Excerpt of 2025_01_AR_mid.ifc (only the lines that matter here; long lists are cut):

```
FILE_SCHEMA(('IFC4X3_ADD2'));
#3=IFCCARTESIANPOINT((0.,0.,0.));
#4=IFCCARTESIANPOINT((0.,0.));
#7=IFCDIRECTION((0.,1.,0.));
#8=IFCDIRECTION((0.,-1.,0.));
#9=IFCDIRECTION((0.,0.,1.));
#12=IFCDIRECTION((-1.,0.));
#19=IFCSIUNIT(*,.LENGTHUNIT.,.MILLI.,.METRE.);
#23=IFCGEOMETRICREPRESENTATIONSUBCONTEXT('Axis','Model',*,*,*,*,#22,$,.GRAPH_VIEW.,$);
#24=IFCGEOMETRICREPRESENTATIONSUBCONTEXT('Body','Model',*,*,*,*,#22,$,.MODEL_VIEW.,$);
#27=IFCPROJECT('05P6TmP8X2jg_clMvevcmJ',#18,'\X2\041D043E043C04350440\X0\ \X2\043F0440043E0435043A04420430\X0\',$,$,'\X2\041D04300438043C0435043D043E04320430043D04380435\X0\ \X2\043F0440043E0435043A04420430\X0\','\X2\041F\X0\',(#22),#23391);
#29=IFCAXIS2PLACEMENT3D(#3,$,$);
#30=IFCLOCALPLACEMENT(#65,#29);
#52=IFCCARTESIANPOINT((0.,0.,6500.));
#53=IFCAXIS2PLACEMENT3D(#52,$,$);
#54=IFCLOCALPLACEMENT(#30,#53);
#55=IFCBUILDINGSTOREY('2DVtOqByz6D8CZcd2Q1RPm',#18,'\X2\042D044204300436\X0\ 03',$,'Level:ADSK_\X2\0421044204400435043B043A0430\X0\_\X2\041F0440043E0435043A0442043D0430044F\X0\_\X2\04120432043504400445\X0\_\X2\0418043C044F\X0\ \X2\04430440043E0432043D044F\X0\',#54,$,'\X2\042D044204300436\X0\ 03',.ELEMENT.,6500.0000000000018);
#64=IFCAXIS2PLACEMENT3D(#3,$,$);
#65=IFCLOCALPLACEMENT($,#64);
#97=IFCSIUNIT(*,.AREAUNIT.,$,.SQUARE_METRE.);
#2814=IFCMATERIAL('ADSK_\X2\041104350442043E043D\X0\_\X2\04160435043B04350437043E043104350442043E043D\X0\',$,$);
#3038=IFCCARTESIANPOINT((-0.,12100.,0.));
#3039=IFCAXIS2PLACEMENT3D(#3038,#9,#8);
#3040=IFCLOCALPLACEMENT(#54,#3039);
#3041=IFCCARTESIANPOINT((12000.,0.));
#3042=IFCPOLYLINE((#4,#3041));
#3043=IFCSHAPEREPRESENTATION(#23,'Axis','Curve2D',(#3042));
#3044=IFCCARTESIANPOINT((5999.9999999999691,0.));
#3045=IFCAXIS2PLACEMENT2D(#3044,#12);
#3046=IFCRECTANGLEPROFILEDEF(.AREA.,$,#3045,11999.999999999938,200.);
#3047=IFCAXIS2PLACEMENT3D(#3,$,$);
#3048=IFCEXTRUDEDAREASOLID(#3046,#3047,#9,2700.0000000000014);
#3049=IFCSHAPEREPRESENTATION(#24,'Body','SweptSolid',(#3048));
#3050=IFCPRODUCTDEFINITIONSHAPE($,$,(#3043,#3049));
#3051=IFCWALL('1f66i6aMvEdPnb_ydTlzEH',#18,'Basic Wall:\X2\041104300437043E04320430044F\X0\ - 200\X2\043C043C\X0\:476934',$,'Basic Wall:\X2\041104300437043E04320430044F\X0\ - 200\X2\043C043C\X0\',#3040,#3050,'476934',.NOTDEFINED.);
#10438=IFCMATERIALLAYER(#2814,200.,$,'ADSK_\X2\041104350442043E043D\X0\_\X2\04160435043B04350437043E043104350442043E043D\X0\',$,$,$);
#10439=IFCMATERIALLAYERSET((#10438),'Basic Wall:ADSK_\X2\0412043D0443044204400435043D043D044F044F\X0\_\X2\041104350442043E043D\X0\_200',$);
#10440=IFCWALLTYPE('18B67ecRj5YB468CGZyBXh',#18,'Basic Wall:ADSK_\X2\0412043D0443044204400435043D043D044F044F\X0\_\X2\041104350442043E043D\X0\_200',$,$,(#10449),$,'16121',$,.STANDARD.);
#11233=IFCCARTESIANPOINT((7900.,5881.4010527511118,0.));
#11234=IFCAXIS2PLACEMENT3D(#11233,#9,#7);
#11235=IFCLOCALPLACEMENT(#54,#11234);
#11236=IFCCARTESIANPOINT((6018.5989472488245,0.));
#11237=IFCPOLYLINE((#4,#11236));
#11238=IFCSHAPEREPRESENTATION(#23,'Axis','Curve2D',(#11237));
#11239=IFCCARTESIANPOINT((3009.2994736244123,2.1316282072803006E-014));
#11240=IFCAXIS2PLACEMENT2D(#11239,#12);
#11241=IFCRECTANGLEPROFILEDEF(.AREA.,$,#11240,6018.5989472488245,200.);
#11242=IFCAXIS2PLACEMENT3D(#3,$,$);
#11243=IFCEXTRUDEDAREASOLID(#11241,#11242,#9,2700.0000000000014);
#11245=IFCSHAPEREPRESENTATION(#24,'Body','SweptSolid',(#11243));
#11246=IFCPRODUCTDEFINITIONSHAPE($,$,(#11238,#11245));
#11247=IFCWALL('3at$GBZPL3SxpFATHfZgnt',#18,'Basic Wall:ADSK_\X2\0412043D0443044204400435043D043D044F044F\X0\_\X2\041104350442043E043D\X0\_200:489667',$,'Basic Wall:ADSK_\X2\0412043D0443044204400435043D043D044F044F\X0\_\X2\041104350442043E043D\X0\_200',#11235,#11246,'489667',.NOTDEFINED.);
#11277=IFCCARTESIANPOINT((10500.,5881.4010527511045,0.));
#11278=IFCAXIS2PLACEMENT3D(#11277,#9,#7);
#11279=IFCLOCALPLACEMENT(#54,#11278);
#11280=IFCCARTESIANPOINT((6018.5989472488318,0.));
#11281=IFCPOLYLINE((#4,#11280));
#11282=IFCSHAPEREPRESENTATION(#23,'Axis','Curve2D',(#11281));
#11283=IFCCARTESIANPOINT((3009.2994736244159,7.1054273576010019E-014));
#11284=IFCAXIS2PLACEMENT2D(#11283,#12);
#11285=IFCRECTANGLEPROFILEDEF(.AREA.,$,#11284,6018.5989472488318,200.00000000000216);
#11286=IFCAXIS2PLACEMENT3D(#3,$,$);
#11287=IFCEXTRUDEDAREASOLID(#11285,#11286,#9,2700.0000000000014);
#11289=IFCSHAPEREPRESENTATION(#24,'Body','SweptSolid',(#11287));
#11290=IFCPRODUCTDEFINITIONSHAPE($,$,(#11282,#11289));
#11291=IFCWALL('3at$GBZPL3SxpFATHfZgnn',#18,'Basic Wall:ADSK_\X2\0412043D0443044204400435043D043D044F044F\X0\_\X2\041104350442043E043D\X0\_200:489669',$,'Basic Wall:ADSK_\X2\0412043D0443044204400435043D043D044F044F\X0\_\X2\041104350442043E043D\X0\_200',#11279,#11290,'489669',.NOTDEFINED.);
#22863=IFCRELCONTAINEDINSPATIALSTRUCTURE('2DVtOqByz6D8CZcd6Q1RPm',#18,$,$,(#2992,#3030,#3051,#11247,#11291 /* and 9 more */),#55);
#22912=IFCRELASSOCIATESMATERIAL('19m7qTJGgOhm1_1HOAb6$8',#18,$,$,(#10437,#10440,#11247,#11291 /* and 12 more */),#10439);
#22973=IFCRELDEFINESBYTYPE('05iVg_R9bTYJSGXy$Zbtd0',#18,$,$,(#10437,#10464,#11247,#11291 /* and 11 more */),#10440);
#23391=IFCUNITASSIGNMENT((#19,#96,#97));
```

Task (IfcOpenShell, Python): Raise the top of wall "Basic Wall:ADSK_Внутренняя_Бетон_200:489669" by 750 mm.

```python
import ifcopenshell
import ifcopenshell.geom
import ifcopenshell.util.representation
import ifcopenshell.util.shape

model = ifcopenshell.open("2025_01_AR_mid.ifc")
settings = ifcopenshell.geom.settings()


def volume(element):
    """Net volume in cubic metres, openings subtracted."""
    shape = ifcopenshell.geom.create_shape(settings, element)
    return ifcopenshell.util.shape.get_volume(shape.geometry)


wall = model.by_id(11291)
before = volume(wall)

body = ifcopenshell.util.representation.get_representation(wall, "Model", "Body")
solid = body.Items[0]
old_height = solid.Depth
solid.Depth += 750.0
after = volume(wall)

print(f"height {old_height:g} -> {solid.Depth:g}, volume {before:.3f} -> {after:.3f} m3")

model.write("2025_01_AR_mid_updated.ifc")
```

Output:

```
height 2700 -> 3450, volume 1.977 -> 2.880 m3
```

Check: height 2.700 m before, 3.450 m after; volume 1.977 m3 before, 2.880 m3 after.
